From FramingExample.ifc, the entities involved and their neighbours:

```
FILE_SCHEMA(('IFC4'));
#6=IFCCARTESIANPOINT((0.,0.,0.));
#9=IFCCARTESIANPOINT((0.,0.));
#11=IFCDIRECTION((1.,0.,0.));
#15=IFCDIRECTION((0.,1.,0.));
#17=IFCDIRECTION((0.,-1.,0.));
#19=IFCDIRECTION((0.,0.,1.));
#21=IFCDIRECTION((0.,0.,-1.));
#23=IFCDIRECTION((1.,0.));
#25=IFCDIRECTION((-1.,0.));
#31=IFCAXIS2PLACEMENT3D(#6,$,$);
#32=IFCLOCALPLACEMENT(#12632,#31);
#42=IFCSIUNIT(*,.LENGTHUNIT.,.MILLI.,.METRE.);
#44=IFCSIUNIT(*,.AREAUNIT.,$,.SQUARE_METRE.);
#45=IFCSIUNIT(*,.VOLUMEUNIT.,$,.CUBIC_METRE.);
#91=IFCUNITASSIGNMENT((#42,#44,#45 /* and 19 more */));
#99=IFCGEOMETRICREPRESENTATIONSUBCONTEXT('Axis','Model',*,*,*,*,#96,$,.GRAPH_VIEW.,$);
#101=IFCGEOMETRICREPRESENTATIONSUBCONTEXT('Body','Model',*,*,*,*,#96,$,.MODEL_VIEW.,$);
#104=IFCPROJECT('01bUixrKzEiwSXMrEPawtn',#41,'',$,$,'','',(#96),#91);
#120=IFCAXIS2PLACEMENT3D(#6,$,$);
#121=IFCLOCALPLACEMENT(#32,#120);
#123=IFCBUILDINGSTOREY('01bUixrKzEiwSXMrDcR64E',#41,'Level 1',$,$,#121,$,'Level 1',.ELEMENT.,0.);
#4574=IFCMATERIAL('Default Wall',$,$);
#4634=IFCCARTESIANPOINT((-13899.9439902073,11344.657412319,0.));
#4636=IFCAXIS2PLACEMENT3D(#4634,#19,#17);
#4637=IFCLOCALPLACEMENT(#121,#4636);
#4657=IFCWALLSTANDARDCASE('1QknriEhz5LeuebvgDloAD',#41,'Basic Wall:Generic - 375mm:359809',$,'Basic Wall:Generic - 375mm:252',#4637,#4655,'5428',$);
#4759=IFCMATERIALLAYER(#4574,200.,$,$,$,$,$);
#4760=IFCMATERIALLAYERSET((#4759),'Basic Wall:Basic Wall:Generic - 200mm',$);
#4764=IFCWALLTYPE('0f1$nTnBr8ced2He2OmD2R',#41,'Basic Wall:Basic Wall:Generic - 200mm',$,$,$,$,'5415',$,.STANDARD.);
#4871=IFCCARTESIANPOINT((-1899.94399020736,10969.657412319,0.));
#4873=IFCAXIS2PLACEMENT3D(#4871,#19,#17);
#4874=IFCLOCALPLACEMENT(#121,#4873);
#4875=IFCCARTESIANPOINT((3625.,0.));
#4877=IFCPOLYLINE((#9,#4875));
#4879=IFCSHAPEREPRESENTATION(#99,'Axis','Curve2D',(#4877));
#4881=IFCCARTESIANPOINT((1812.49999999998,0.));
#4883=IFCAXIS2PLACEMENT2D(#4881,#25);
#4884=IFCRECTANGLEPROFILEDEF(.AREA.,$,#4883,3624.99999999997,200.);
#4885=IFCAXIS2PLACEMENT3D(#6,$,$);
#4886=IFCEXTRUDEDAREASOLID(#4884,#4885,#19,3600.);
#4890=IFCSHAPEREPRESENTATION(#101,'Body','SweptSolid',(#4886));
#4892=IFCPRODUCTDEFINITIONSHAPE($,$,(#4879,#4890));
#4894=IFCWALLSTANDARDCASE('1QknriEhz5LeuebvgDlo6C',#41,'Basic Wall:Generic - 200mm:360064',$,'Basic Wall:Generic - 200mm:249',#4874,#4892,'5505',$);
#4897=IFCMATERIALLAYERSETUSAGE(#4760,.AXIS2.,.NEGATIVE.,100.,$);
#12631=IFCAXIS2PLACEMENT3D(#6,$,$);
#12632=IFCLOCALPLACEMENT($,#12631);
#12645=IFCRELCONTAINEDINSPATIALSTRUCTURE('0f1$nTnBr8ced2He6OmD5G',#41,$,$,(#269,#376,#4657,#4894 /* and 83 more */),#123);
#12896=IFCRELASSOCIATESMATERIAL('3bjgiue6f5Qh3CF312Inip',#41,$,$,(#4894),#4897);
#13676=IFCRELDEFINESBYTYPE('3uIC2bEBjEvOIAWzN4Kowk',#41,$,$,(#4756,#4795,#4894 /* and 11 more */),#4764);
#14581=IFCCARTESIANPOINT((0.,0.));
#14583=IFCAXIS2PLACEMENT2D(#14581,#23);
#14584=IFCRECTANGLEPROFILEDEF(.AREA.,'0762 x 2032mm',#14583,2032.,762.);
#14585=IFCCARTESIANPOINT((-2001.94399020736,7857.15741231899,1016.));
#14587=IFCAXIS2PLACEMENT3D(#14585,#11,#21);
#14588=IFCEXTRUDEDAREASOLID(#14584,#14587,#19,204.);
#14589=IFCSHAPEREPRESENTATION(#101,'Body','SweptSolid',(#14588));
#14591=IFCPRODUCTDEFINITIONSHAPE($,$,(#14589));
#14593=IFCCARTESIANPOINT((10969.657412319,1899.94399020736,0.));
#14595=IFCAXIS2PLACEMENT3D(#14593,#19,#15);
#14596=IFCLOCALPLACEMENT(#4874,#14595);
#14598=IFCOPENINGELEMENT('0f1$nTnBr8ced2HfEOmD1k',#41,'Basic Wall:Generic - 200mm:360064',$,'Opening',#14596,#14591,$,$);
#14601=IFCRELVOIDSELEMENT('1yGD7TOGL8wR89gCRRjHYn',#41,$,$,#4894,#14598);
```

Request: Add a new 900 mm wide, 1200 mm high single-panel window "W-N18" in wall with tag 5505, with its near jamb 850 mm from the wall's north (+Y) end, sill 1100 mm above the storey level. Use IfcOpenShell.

```python
import numpy as np
import ifcopenshell
import ifcopenshell.api.feature
import ifcopenshell.api.geometry
import ifcopenshell.api.root
import ifcopenshell.api.spatial
import ifcopenshell.geom
import ifcopenshell.util.element
import ifcopenshell.util.placement
import ifcopenshell.util.representation
import ifcopenshell.util.shape
import ifcopenshell.util.unit

model = ifcopenshell.open("FramingExample.ifc")
unit_scale = ifcopenshell.util.unit.calculate_unit_scale(model)
settings = ifcopenshell.geom.settings()


def volume(element):
    """Net volume in cubic metres, openings subtracted."""
    shape = ifcopenshell.geom.create_shape(settings, element)
    return ifcopenshell.util.shape.get_volume(shape.geometry)


wall = model.by_guid("1QknriEhz5LeuebvgDlo6C")
storey = ifcopenshell.util.element.get_container(wall, ifc_class="IfcBuildingStorey")
context = ifcopenshell.util.representation.get_context(model, "Model", "Body", "MODEL_VIEW")
before = volume(wall)

width, height, from_end, sill = 0.9, 1.2, 0.85, 1.1  # metres

# The wall runs along its own X axis, and the end named is its -X end.
wall_shape = ifcopenshell.geom.create_shape(settings, wall)
x, y, z = ifcopenshell.util.shape.get_vertices(wall_shape.geometry).T
start = x.min() + from_end
face, thickness = float(y.min()), float(y.max() - y.min())
wall_matrix = ifcopenshell.util.placement.get_local_placement(wall.ObjectPlacement)
level = ifcopenshell.util.placement.get_local_placement(storey.ObjectPlacement)[2, 3]


def in_wall(x, y):
    """Placement at x, y metres in the wall's axes, at sill height."""
    matrix = wall_matrix.copy()
    matrix[:, 3] = wall_matrix @ np.array([x / unit_scale, y / unit_scale, 0.0, 1.0])
    matrix[2, 3] = level + sill / unit_scale
    return matrix


# Opening: a box that overshoots both wall faces by 50 mm.
opening = ifcopenshell.api.root.create_entity(model, ifc_class="IfcOpeningElement", predefined_type="OPENING")
box = ifcopenshell.api.geometry.add_wall_representation(
    model, context=context, length=width, height=height, thickness=thickness + 0.1
)
ifcopenshell.api.geometry.assign_representation(model, product=opening, representation=box)
ifcopenshell.api.geometry.edit_object_placement(model, product=opening, matrix=in_wall(start, face - 0.05), is_si=False)
ifcopenshell.api.feature.add_feature(model, feature=opening, element=wall)

window = ifcopenshell.api.root.create_entity(model, ifc_class="IfcWindow", name="W-N18", predefined_type="WINDOW")
window.OverallWidth, window.OverallHeight = width / unit_scale, height / unit_scale
window.PartitioningType = "SINGLE_PANEL"
body = ifcopenshell.api.geometry.add_window_representation(
    model,
    context=context,
    overall_width=window.OverallWidth,
    overall_height=window.OverallHeight,
    partition_type="SINGLE_PANEL",
)
ifcopenshell.api.geometry.assign_representation(model, product=window, representation=body)
ifcopenshell.api.spatial.assign_container(model, products=[window], relating_structure=storey)
ifcopenshell.api.feature.add_filling(model, opening=opening, element=window)

# Centre the window in the wall's thickness.
ifcopenshell.api.geometry.edit_object_placement(model, product=window, matrix=in_wall(start, face), is_si=False)
window_shape = ifcopenshell.geom.create_shape(settings, window)
depth = ifcopenshell.util.shape.get_vertices(window_shape.geometry)[:, 1]
offset = face + thickness / 2 - (depth.min() + depth.max()) / 2
ifcopenshell.api.geometry.edit_object_placement(model, product=window, matrix=in_wall(start, offset), is_si=False)

after = volume(wall)

print(f"wall volume {before:.3f} -> {after:.3f} m3")

model.write("FramingExample_edited.ifc")
```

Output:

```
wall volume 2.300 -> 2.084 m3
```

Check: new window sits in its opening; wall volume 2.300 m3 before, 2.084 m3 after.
